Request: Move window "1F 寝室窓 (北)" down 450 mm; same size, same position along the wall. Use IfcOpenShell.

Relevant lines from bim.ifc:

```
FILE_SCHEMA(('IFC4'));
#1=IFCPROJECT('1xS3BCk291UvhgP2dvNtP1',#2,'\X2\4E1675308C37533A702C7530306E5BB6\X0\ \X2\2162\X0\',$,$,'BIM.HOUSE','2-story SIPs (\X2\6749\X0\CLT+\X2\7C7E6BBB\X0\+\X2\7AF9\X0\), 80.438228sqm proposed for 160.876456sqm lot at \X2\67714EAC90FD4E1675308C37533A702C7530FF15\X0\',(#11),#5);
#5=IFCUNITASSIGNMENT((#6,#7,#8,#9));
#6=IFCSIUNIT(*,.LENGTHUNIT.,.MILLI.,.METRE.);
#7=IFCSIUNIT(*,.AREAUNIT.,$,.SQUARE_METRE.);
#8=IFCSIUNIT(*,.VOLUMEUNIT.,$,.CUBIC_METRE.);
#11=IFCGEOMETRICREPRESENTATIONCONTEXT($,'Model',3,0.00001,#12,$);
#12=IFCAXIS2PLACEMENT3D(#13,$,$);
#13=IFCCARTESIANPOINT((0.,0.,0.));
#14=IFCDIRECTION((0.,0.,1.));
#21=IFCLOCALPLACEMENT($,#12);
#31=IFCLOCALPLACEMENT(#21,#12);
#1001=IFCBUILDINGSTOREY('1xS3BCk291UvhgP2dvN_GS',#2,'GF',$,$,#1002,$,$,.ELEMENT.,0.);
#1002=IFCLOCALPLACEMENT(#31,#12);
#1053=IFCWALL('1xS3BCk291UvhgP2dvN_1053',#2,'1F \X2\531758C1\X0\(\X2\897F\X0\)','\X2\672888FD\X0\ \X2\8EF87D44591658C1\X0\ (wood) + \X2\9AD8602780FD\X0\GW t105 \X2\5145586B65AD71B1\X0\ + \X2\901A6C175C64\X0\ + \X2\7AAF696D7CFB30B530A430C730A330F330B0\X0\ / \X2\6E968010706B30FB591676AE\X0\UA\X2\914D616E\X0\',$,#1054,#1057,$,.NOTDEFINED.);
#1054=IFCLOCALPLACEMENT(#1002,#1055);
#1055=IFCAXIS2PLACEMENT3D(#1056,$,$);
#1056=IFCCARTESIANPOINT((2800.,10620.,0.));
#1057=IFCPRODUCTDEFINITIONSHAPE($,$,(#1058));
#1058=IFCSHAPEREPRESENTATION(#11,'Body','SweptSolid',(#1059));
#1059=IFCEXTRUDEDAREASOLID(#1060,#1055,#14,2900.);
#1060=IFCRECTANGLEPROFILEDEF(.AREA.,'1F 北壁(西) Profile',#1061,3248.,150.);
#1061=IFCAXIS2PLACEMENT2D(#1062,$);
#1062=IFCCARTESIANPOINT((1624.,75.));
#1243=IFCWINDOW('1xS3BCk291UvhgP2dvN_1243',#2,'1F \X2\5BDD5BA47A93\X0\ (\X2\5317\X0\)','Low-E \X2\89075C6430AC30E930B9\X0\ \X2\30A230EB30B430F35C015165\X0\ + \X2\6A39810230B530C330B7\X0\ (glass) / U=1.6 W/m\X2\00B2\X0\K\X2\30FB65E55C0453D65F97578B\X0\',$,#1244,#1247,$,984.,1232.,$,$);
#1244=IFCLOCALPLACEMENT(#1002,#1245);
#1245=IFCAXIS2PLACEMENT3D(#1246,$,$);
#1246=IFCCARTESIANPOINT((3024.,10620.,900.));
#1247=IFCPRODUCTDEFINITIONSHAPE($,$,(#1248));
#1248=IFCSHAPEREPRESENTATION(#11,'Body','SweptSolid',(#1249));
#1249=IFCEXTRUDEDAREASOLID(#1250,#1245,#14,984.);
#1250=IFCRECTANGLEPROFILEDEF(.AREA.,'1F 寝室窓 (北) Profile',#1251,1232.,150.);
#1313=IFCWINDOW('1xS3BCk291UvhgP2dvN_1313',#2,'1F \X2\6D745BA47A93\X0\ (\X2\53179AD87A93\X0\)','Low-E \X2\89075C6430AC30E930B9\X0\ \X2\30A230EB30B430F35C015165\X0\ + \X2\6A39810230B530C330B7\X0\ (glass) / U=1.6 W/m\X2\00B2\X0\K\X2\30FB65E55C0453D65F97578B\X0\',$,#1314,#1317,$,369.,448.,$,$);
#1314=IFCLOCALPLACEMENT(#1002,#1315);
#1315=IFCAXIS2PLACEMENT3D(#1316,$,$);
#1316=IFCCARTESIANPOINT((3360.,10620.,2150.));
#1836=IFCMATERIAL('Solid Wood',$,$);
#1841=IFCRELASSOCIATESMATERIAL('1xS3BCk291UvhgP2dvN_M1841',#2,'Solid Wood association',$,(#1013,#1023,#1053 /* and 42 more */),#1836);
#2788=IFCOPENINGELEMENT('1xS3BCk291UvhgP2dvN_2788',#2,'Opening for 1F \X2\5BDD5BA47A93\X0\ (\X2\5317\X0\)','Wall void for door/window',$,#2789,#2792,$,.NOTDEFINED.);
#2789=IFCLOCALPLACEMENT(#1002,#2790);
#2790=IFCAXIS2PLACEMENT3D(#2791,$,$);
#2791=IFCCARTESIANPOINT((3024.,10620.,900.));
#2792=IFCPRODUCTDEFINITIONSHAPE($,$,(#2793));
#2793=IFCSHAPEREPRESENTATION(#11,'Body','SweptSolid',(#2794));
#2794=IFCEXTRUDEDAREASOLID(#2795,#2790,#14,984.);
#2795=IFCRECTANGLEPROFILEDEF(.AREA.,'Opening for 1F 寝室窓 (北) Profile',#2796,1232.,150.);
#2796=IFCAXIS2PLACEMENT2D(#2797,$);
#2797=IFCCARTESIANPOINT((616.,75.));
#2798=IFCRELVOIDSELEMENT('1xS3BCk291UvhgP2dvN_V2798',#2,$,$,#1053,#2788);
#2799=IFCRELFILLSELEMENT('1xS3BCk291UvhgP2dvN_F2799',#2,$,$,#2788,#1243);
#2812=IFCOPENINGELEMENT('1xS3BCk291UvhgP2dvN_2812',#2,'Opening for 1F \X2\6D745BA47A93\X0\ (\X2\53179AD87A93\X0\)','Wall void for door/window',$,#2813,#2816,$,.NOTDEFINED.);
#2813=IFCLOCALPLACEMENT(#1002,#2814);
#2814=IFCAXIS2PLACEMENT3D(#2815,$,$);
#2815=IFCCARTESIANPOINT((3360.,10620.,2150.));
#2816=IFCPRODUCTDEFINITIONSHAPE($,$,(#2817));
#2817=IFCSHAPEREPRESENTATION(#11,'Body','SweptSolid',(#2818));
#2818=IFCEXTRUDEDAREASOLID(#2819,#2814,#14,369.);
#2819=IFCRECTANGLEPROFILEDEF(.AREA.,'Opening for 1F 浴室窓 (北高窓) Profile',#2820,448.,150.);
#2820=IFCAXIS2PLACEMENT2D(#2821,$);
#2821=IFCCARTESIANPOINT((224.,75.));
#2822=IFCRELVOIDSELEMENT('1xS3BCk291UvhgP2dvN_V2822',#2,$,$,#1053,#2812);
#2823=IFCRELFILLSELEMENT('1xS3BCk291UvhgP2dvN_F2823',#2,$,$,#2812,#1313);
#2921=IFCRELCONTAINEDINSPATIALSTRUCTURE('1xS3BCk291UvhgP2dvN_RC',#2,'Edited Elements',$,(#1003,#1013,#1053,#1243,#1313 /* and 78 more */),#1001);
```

```python
import numpy as np
import ifcopenshell
import ifcopenshell.api.geometry
import ifcopenshell.util.placement
import ifcopenshell.util.unit

model = ifcopenshell.open("bim.ifc")
unit_scale = ifcopenshell.util.unit.calculate_unit_scale(model)

window = model.by_id(1243)
opening = window.FillsVoids[0].RelatingOpeningElement
dz = -0.45 / unit_scale

shift = np.array([0.0, 0.0, dz])
# The window is not placed relative to its opening, so move both.
for product in (opening, window):
    matrix = ifcopenshell.util.placement.get_local_placement(product.ObjectPlacement)
    matrix[:3, 3] += shift
    ifcopenshell.api.geometry.edit_object_placement(model, product=product, matrix=matrix, is_si=False)

print(f"moved by {dz * unit_scale:+.3f} m")

model.write("bim-out.ifc")
```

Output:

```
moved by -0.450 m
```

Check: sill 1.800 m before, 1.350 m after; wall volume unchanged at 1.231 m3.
